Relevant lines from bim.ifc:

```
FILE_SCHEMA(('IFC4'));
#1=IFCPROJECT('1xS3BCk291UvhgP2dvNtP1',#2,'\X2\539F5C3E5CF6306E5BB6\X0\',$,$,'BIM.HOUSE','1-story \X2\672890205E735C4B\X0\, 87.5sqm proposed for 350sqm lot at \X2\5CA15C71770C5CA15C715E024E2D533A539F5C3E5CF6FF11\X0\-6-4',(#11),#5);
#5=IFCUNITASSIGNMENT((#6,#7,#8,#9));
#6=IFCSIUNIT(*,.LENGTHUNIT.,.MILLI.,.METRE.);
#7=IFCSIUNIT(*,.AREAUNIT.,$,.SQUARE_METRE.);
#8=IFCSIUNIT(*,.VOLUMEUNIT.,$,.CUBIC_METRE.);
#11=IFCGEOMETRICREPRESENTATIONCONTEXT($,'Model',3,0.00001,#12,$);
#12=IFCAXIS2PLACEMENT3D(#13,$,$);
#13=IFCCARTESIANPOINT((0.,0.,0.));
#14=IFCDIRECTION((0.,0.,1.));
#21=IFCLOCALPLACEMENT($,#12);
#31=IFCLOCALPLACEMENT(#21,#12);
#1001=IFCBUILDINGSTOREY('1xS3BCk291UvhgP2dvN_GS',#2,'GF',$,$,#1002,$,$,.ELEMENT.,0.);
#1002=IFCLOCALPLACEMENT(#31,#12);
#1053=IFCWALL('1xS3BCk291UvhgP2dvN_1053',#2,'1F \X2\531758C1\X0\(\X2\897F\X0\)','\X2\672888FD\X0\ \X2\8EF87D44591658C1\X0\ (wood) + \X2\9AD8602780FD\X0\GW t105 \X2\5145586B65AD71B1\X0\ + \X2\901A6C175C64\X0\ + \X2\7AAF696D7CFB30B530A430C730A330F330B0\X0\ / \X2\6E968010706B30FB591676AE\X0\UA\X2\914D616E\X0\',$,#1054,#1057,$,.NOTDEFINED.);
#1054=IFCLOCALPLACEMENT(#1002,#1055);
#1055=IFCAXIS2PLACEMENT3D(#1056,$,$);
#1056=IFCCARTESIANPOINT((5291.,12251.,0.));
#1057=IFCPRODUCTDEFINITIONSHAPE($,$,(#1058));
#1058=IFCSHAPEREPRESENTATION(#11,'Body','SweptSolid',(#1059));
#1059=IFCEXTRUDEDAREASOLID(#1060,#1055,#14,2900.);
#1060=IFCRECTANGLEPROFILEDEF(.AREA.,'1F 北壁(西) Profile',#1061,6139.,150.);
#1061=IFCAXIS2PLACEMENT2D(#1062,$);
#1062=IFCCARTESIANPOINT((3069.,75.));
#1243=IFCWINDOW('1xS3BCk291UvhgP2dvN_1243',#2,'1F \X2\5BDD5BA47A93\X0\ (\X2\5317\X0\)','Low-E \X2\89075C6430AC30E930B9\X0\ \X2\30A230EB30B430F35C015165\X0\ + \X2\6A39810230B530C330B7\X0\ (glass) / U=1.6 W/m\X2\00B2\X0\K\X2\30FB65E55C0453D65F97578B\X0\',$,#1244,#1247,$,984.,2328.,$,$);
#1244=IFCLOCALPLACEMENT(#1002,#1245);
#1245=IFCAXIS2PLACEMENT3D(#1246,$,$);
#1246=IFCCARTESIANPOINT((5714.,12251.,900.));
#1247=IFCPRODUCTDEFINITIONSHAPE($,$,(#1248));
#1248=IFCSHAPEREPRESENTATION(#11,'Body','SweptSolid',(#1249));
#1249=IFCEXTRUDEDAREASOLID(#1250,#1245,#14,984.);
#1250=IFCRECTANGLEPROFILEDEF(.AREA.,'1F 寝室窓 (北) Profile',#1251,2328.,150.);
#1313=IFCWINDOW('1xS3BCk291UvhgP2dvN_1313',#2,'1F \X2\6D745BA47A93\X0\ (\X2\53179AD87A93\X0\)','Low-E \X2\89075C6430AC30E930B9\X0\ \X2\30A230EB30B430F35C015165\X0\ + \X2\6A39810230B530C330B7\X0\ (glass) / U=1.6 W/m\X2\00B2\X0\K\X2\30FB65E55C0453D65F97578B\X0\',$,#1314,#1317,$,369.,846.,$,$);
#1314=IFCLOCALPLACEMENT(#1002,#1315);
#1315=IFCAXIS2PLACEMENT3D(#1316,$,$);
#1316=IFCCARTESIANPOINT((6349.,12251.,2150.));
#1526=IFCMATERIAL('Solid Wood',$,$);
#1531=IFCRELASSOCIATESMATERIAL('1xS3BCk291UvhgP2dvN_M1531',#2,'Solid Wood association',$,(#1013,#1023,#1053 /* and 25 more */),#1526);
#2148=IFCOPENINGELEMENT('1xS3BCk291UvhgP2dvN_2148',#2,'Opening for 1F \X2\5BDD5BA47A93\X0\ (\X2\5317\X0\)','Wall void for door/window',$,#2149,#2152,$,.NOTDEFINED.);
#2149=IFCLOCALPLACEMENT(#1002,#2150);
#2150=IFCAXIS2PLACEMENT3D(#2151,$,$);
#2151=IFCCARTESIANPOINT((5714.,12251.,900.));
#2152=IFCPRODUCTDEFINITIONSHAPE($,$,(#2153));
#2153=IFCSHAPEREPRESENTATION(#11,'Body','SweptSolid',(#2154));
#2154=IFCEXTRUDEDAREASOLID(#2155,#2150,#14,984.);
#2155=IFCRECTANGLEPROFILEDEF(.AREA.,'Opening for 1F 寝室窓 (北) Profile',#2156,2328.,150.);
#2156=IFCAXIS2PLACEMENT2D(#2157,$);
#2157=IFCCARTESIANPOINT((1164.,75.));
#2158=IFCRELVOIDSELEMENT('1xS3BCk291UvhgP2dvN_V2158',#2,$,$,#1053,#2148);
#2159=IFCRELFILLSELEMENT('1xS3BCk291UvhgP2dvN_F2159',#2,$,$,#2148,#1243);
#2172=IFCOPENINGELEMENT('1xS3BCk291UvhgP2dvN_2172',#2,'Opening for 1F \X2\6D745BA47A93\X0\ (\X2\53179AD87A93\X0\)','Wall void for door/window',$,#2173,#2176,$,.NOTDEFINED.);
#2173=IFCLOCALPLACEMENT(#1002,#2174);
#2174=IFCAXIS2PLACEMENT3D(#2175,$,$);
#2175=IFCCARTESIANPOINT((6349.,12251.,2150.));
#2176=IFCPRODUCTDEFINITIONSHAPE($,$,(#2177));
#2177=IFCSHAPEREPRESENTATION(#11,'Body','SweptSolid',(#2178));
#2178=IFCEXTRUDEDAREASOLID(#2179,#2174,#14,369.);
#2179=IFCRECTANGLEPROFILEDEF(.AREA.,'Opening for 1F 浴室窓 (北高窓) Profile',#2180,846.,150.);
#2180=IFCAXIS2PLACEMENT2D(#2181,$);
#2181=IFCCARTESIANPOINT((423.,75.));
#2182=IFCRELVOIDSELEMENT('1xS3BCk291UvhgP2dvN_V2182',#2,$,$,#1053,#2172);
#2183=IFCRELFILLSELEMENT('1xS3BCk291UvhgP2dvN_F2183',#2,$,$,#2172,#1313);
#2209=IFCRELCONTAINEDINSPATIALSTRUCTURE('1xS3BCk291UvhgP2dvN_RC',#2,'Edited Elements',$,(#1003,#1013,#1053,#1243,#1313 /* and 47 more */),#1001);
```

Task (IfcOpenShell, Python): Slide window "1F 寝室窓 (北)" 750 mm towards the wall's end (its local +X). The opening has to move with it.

```python
import ifcopenshell
import ifcopenshell.api.geometry
import ifcopenshell.util.placement

model = ifcopenshell.open("bim.ifc")

window = model.by_guid("1xS3BCk291UvhgP2dvN_1243")
opening = window.FillsVoids[0].RelatingOpeningElement
wall = opening.VoidsElements[0].RelatingBuildingElement

wall_matrix = ifcopenshell.util.placement.get_local_placement(wall.ObjectPlacement)
shift = wall_matrix[:3, 0] * 750.0
before = ifcopenshell.util.placement.get_local_placement(window.ObjectPlacement)[:3, 3].copy()

# The window is not placed relative to its opening, so move both.
for product in (opening, window):
    matrix = ifcopenshell.util.placement.get_local_placement(product.ObjectPlacement)
    matrix[:3, 3] += shift
    ifcopenshell.api.geometry.edit_object_placement(model, product=product, matrix=matrix, is_si=False)

after = ifcopenshell.util.placement.get_local_placement(window.ObjectPlacement)[:3, 3]
print("window moved by", (after - before).round(3) + 0.0)

model.write("bim_v2.ifc")
```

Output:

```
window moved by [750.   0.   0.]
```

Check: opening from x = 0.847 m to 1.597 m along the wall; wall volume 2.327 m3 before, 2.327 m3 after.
